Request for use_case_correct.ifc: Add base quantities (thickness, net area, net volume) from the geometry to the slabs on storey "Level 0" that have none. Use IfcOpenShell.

First a look at what the model holds.

```python
import ifcopenshell
import ifcopenshell.util.element
import ifcopenshell.util.unit

model = ifcopenshell.open("use_case_correct.ifc")
print(model.schema)
for unit_type in ("LENGTHUNIT", "AREAUNIT", "VOLUMEUNIT"):
    print(unit_type, ifcopenshell.util.unit.calculate_unit_scale(model, unit_type))
storey = next(s for s in model.by_type("IfcBuildingStorey") if s.Name == "Level 0")
slabs = [e for e in ifcopenshell.util.element.get_decomposition(storey) if e.is_a("IfcSlab")]
for e in sorted(slabs, key=lambda e: e.id()):
    print(e.id(), e.is_a(), e.Name, list(ifcopenshell.util.element.get_psets(e, qtos_only=True)), sep=" | ")
```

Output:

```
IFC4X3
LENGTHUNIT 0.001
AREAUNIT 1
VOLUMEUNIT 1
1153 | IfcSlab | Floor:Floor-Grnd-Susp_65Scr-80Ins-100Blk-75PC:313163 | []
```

```python
import ifcopenshell
import ifcopenshell.api.pset
import ifcopenshell.geom
import ifcopenshell.util.element
import ifcopenshell.util.shape
import ifcopenshell.util.unit

model = ifcopenshell.open("use_case_correct.ifc")
unit_scale = ifcopenshell.util.unit.calculate_unit_scale(model)
area_scale = ifcopenshell.util.unit.calculate_unit_scale(model, "AREAUNIT")
volume_scale = ifcopenshell.util.unit.calculate_unit_scale(model, "VOLUMEUNIT")
settings = ifcopenshell.geom.settings()

storey = next(s for s in model.by_type("IfcBuildingStorey") if s.Name == "Level 0")
slabs = [e for e in ifcopenshell.util.element.get_decomposition(storey) if e.is_a("IfcSlab")]

for e in sorted(slabs, key=lambda e: e.id()):
    if ifcopenshell.util.element.get_psets(e, qtos_only=True, should_inherit=False):
        continue
    # Geometry comes back in metres, in the element's own axes.
    shape = ifcopenshell.geom.create_shape(settings, e)
    values = {
        "Width": ifcopenshell.util.shape.get_z(shape.geometry) / unit_scale,
        "NetArea": ifcopenshell.util.shape.get_footprint_area(shape.geometry) / area_scale,
        "NetVolume": ifcopenshell.util.shape.get_volume(shape.geometry) / volume_scale,
    }
    qto = ifcopenshell.api.pset.add_qto(model, product=e, name="Qto_SlabBaseQuantities")
    ifcopenshell.api.pset.edit_qto(model, qto=qto, properties=values)
    print(e.id(), {k: round(v, 3) for k, v in values.items()})

model.write("use_case_correct_updated.ifc")
```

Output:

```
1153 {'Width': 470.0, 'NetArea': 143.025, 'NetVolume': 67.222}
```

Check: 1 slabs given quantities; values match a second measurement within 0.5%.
